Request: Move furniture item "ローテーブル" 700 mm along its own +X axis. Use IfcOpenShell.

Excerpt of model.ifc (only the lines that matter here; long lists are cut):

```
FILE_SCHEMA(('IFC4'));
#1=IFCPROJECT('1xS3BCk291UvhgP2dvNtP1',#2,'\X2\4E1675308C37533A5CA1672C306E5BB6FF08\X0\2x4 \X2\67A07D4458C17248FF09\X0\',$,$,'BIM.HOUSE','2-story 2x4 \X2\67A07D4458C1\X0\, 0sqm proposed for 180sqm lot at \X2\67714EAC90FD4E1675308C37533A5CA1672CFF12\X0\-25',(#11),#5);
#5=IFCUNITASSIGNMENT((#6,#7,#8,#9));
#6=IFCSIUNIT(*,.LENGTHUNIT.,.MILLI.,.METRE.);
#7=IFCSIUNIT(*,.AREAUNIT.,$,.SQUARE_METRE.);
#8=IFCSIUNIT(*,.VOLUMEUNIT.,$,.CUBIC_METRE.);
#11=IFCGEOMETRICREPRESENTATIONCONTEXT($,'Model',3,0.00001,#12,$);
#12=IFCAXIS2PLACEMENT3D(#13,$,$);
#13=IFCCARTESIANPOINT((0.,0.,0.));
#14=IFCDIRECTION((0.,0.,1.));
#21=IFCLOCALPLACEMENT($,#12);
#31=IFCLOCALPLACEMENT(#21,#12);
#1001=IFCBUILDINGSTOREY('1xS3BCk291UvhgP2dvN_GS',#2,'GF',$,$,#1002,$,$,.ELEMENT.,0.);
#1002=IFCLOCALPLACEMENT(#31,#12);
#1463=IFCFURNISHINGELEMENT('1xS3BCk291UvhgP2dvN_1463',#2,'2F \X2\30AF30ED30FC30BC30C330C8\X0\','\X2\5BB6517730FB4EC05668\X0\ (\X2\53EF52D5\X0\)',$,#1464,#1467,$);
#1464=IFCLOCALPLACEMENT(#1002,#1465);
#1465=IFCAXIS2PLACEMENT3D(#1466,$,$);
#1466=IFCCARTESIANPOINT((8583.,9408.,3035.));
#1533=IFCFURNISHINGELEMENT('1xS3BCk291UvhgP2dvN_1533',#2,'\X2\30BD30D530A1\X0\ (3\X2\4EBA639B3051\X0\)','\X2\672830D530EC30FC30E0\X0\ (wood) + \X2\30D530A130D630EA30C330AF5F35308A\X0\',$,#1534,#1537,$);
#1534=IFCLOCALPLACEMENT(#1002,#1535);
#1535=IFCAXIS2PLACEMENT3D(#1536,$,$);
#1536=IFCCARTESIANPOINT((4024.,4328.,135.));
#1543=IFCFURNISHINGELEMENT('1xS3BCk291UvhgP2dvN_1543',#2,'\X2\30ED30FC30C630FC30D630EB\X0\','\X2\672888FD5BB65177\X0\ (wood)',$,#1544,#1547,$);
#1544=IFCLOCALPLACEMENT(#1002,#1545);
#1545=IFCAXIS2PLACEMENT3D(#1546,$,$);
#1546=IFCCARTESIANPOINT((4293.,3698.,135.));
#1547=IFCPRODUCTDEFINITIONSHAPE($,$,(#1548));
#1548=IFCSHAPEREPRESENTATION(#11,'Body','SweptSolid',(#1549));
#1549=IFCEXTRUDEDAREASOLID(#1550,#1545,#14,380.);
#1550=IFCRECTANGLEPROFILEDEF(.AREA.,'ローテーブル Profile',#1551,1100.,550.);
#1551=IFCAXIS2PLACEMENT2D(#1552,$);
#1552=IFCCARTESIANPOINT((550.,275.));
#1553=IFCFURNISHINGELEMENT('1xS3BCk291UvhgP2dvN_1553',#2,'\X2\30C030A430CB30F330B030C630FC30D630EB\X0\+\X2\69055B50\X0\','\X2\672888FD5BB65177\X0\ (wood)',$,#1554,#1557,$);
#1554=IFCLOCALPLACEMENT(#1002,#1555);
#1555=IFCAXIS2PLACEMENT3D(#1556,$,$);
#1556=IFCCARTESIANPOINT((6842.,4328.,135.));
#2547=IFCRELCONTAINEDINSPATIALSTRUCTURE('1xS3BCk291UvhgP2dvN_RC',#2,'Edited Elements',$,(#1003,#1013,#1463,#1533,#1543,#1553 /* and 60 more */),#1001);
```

```python
import ifcopenshell
import ifcopenshell.api.geometry
import ifcopenshell.util.placement
import ifcopenshell.util.unit

model = ifcopenshell.open("model.ifc")
unit_scale = ifcopenshell.util.unit.calculate_unit_scale(model)

item = model.by_guid("1xS3BCk291UvhgP2dvN_1543")
matrix = ifcopenshell.util.placement.get_local_placement(item.ObjectPlacement)
matrix[:3, 3] += matrix[:3, 0] * 0.7 / unit_scale
ifcopenshell.api.geometry.edit_object_placement(model, product=item, matrix=matrix, is_si=False)

print(ifcopenshell.util.placement.get_local_placement(item.ObjectPlacement).round(3) + 0.0)

model.write("model_edited.ifc")
```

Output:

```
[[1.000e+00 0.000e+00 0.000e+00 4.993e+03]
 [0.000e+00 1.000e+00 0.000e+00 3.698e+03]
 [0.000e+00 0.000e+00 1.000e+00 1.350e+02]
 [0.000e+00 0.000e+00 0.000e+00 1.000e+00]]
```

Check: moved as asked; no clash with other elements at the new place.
